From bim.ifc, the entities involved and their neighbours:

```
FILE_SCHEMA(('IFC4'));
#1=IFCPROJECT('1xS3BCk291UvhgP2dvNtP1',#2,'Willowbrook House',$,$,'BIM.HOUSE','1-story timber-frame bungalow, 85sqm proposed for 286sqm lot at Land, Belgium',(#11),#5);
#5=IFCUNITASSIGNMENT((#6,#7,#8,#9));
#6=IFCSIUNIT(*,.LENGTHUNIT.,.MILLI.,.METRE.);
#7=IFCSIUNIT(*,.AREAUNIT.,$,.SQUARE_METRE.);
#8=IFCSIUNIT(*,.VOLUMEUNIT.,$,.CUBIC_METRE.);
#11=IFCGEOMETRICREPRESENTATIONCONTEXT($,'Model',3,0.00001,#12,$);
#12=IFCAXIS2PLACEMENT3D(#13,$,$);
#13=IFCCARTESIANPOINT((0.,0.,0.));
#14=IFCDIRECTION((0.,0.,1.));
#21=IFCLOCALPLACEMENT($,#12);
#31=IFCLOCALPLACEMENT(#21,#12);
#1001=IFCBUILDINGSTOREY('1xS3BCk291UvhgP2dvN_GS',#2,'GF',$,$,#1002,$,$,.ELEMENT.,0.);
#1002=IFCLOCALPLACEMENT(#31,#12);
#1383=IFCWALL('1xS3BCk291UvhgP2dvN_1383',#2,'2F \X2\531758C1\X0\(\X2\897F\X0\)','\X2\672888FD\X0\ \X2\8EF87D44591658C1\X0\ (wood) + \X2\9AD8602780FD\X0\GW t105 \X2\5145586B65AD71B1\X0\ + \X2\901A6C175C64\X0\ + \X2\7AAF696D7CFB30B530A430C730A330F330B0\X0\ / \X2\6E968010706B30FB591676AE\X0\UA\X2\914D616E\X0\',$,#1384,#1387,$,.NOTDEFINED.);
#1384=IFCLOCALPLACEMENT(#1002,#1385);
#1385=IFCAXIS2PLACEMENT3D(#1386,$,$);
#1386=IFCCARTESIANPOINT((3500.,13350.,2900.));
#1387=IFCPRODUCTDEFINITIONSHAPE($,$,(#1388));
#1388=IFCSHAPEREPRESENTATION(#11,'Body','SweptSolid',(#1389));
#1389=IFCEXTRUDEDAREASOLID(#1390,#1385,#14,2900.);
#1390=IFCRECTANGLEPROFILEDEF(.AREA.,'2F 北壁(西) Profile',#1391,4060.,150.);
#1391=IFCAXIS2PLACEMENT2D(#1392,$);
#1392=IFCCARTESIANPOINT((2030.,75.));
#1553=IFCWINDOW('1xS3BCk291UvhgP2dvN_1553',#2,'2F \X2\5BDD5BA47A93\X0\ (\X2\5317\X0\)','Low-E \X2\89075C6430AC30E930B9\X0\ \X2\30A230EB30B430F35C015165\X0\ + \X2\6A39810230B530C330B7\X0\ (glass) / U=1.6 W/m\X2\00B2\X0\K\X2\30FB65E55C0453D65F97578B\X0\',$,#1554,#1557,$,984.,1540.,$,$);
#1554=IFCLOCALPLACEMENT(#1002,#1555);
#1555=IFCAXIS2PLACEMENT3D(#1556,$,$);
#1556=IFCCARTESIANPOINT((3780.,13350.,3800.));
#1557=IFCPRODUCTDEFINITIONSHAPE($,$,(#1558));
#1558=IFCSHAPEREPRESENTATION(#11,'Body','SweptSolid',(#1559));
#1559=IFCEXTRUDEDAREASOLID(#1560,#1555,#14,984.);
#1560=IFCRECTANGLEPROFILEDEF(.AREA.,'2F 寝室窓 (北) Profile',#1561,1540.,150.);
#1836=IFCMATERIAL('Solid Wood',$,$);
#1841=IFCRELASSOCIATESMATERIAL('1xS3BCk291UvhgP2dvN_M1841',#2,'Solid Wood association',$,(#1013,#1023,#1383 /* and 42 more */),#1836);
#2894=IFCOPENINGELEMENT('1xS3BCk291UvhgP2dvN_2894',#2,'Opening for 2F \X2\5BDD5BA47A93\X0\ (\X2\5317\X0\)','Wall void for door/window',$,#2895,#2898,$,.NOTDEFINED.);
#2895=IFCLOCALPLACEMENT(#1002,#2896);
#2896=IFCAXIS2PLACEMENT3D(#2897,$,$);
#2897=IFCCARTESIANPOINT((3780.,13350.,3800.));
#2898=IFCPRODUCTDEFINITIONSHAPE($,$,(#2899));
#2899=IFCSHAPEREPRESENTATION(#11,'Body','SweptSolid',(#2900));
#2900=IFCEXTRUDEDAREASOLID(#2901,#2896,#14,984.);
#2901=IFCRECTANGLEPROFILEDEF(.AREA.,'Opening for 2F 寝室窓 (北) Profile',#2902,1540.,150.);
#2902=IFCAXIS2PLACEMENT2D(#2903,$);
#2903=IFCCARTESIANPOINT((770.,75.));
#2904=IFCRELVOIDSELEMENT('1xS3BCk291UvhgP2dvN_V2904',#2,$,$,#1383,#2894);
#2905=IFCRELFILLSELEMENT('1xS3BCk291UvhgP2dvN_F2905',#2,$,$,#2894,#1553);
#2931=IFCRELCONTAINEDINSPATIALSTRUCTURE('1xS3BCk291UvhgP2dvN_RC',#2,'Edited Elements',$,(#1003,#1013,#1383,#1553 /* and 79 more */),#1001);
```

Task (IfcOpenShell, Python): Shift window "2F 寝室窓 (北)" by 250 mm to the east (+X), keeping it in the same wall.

```python
import ifcopenshell
import ifcopenshell.api.geometry
import ifcopenshell.util.placement
import ifcopenshell.util.unit

model = ifcopenshell.open("bim.ifc")
unit_scale = ifcopenshell.util.unit.calculate_unit_scale(model)

window = model.by_id(1553)
opening = window.FillsVoids[0].RelatingOpeningElement
wall = opening.VoidsElements[0].RelatingBuildingElement

wall_matrix = ifcopenshell.util.placement.get_local_placement(wall.ObjectPlacement)
shift = wall_matrix[:3, 0] * 0.25 / unit_scale
before = ifcopenshell.util.placement.get_local_placement(window.ObjectPlacement)[:3, 3].copy()

# The window is not placed relative to its opening, so move both.
for product in (opening, window):
    matrix = ifcopenshell.util.placement.get_local_placement(product.ObjectPlacement)
    matrix[:3, 3] += shift
    ifcopenshell.api.geometry.edit_object_placement(model, product=product, matrix=matrix, is_si=False)

after = ifcopenshell.util.placement.get_local_placement(window.ObjectPlacement)[:3, 3]
print("window moved by", (after - before).round(3) + 0.0)

model.write("bim-out.ifc")
```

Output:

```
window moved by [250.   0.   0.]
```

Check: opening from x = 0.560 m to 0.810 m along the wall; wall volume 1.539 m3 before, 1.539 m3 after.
